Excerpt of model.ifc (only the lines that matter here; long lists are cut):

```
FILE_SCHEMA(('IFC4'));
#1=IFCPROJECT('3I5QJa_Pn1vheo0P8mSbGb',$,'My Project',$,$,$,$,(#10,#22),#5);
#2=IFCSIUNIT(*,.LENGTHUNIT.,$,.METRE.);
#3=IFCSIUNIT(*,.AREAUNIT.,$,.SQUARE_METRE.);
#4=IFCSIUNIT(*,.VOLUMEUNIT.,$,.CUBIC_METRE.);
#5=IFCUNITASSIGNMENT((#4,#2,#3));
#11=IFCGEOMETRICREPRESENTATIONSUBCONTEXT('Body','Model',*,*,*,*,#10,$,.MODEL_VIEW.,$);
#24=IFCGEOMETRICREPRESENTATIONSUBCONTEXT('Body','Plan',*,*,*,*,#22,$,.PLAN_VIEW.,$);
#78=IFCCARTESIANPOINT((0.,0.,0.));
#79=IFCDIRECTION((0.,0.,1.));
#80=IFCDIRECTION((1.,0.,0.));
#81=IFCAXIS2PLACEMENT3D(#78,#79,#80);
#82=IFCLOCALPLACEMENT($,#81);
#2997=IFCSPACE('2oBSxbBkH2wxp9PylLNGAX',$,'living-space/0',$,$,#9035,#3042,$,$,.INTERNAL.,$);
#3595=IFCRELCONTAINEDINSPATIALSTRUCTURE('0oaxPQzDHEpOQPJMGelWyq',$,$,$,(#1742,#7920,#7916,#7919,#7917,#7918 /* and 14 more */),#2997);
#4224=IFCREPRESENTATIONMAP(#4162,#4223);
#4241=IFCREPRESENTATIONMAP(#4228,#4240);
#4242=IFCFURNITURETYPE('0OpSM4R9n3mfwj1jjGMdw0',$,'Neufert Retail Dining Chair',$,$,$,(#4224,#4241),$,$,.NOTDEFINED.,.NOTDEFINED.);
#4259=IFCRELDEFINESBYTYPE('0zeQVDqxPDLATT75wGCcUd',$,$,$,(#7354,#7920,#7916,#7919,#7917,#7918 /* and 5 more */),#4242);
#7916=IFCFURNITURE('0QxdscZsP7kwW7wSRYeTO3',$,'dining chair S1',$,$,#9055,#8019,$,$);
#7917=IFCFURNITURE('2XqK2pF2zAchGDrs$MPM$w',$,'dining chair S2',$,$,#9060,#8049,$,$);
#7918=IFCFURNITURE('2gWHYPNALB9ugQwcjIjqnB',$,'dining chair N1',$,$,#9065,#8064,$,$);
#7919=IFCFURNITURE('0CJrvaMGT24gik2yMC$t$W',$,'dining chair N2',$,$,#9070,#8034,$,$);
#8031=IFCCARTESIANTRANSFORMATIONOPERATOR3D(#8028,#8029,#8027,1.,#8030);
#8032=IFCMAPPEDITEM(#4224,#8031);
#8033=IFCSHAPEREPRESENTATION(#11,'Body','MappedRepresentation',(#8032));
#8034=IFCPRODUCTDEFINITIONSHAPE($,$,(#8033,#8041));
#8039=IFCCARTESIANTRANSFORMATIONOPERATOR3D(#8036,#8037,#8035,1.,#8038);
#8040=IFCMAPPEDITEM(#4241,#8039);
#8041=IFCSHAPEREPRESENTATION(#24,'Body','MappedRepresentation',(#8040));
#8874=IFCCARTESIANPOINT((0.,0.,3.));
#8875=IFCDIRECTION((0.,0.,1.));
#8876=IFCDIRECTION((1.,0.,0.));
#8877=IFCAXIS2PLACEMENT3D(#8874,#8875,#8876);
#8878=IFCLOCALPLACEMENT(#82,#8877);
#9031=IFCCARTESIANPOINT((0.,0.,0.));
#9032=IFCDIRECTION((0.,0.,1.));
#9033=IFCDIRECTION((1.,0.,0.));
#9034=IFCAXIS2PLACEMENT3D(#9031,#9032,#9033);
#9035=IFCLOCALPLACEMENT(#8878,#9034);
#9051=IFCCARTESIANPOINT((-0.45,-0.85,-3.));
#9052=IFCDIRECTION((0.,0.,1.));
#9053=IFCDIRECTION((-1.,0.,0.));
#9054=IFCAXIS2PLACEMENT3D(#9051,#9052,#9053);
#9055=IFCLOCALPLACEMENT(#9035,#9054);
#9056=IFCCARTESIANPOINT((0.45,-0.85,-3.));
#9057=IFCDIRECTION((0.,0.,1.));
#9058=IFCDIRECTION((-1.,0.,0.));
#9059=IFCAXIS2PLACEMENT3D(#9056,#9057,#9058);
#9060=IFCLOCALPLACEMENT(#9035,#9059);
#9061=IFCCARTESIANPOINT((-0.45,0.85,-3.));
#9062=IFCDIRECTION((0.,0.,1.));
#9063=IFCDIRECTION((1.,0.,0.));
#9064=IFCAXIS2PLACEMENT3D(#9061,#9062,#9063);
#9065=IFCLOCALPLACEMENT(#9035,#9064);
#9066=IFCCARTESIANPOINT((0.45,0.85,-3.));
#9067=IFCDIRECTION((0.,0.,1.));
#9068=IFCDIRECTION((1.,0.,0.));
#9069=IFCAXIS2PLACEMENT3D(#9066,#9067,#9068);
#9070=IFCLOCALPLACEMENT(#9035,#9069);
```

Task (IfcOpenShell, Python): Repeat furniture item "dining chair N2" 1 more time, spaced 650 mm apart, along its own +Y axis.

```python
import ifcopenshell
import ifcopenshell.api.geometry
import ifcopenshell.api.root
import ifcopenshell.util.element
import ifcopenshell.util.placement
import ifcopenshell.util.unit

model = ifcopenshell.open("model.ifc")
unit_scale = ifcopenshell.util.unit.calculate_unit_scale(model)

source = model.by_guid("0CJrvaMGT24gik2yMC$t$W")
base = ifcopenshell.util.placement.get_local_placement(source.ObjectPlacement)
step = base[:3, 1] * 0.65 / unit_scale

for i in range(1, 2):
    copy = ifcopenshell.api.root.copy_class(model, product=source)
    copy.Representation = ifcopenshell.util.element.copy_deep(
        model, source.Representation, exclude=["IfcGeometricRepresentationContext", "IfcRepresentationMap"]
    )
    matrix = base.copy()
    matrix[:3, 3] += i * step
    print("added at", matrix[:3, 3].round(3) + 0.0)
    ifcopenshell.api.geometry.edit_object_placement(model, product=copy, matrix=matrix, is_si=False)

model.write("model_v2.ifc")
```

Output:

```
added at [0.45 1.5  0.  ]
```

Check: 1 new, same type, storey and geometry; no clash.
